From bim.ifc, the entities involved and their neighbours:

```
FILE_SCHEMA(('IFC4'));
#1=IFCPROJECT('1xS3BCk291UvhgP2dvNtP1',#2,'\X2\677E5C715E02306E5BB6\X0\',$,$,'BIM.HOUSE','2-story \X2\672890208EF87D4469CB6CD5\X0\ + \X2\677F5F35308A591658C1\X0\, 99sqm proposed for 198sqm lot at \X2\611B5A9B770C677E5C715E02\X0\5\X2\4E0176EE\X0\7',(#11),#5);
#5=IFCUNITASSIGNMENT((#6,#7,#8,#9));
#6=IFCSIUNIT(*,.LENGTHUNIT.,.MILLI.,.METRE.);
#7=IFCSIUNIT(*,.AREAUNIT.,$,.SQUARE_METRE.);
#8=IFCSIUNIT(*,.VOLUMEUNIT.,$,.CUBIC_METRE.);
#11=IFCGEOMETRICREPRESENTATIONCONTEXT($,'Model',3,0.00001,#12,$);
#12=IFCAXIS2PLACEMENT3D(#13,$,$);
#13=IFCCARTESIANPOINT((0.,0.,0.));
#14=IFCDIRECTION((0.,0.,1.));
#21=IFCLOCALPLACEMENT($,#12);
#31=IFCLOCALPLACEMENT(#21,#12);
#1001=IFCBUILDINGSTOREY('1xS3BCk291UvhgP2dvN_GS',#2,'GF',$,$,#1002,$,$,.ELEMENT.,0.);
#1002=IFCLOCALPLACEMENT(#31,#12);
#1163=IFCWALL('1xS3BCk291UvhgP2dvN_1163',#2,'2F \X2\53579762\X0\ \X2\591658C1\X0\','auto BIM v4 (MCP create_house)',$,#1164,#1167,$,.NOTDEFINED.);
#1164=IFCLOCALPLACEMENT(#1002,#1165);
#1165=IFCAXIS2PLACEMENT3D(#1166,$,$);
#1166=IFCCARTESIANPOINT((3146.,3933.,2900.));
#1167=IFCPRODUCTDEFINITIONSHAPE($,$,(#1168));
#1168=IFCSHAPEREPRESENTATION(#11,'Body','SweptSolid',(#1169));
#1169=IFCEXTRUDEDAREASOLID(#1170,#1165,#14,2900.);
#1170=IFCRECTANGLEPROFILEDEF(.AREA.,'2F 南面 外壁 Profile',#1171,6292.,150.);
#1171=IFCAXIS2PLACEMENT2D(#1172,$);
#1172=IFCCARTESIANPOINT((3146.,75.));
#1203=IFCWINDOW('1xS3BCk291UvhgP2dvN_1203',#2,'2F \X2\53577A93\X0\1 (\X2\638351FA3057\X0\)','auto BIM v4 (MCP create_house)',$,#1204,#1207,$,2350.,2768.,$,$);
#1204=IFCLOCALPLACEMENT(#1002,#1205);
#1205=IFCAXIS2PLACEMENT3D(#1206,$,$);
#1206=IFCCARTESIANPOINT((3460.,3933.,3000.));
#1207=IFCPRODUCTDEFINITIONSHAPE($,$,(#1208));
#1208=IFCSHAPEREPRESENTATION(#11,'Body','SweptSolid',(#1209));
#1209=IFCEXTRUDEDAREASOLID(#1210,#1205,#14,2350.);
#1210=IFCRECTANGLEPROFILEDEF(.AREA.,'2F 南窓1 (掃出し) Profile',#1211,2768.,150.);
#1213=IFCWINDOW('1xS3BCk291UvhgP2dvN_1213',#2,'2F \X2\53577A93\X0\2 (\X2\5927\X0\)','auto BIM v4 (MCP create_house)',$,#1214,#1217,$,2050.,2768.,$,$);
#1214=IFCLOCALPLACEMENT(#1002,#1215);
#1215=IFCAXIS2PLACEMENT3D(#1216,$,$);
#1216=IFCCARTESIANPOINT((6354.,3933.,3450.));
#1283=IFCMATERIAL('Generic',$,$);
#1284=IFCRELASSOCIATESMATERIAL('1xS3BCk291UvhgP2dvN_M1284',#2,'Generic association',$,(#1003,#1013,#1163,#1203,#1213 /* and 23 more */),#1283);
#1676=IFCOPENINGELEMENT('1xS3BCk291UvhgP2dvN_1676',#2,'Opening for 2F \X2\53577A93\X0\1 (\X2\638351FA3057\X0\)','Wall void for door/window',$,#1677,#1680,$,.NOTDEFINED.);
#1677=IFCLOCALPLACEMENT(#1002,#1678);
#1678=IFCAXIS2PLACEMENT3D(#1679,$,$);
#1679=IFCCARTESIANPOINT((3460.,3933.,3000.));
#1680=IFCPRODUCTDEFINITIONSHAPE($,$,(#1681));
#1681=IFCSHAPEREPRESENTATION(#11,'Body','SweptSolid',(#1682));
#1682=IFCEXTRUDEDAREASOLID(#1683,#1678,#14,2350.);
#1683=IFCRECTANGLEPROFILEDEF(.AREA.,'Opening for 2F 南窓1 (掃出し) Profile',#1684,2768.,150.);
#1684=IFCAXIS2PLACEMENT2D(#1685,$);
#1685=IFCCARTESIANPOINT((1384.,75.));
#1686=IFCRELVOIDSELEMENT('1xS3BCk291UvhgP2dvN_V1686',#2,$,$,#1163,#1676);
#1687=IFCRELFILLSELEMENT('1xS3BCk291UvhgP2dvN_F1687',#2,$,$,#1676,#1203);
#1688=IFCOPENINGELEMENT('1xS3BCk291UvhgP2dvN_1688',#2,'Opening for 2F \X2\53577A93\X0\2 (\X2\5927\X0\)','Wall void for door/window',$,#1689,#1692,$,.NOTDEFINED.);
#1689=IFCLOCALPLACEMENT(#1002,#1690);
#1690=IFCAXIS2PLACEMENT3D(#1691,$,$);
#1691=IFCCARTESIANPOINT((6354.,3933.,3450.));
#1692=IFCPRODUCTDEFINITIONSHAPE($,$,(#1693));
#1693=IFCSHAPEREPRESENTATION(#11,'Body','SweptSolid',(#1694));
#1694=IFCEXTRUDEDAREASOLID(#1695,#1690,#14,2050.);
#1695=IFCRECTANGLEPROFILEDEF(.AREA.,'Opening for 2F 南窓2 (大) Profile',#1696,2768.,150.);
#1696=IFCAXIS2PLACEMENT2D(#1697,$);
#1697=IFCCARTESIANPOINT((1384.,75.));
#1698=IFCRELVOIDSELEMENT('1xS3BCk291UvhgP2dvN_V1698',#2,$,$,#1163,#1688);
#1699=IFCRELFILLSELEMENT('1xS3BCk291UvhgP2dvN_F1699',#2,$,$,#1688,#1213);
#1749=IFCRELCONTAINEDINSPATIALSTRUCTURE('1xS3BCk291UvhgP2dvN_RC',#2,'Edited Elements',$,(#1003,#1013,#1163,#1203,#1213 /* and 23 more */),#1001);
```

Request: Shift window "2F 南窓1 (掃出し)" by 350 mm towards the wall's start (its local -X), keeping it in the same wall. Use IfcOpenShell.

```python
import ifcopenshell
import ifcopenshell.api.geometry
import ifcopenshell.util.placement
import ifcopenshell.util.unit

model = ifcopenshell.open("bim.ifc")
unit_scale = ifcopenshell.util.unit.calculate_unit_scale(model)

window = model.by_guid("1xS3BCk291UvhgP2dvN_1203")
opening = window.FillsVoids[0].RelatingOpeningElement
wall = opening.VoidsElements[0].RelatingBuildingElement

wall_matrix = ifcopenshell.util.placement.get_local_placement(wall.ObjectPlacement)
shift = wall_matrix[:3, 0] * -0.35 / unit_scale
before = ifcopenshell.util.placement.get_local_placement(window.ObjectPlacement)[:3, 3].copy()

# The window is not placed relative to its opening, so move both.
for product in (opening, window):
    matrix = ifcopenshell.util.placement.get_local_placement(product.ObjectPlacement)
    matrix[:3, 3] += shift
    ifcopenshell.api.geometry.edit_object_placement(model, product=product, matrix=matrix, is_si=False)

after = ifcopenshell.util.placement.get_local_placement(window.ObjectPlacement)[:3, 3]
print("window moved by", (after - before).round(3) + 0.0)

model.write("bim_updated.ifc")
```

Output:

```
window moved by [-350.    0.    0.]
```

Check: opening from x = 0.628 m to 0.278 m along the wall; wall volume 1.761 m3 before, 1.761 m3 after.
